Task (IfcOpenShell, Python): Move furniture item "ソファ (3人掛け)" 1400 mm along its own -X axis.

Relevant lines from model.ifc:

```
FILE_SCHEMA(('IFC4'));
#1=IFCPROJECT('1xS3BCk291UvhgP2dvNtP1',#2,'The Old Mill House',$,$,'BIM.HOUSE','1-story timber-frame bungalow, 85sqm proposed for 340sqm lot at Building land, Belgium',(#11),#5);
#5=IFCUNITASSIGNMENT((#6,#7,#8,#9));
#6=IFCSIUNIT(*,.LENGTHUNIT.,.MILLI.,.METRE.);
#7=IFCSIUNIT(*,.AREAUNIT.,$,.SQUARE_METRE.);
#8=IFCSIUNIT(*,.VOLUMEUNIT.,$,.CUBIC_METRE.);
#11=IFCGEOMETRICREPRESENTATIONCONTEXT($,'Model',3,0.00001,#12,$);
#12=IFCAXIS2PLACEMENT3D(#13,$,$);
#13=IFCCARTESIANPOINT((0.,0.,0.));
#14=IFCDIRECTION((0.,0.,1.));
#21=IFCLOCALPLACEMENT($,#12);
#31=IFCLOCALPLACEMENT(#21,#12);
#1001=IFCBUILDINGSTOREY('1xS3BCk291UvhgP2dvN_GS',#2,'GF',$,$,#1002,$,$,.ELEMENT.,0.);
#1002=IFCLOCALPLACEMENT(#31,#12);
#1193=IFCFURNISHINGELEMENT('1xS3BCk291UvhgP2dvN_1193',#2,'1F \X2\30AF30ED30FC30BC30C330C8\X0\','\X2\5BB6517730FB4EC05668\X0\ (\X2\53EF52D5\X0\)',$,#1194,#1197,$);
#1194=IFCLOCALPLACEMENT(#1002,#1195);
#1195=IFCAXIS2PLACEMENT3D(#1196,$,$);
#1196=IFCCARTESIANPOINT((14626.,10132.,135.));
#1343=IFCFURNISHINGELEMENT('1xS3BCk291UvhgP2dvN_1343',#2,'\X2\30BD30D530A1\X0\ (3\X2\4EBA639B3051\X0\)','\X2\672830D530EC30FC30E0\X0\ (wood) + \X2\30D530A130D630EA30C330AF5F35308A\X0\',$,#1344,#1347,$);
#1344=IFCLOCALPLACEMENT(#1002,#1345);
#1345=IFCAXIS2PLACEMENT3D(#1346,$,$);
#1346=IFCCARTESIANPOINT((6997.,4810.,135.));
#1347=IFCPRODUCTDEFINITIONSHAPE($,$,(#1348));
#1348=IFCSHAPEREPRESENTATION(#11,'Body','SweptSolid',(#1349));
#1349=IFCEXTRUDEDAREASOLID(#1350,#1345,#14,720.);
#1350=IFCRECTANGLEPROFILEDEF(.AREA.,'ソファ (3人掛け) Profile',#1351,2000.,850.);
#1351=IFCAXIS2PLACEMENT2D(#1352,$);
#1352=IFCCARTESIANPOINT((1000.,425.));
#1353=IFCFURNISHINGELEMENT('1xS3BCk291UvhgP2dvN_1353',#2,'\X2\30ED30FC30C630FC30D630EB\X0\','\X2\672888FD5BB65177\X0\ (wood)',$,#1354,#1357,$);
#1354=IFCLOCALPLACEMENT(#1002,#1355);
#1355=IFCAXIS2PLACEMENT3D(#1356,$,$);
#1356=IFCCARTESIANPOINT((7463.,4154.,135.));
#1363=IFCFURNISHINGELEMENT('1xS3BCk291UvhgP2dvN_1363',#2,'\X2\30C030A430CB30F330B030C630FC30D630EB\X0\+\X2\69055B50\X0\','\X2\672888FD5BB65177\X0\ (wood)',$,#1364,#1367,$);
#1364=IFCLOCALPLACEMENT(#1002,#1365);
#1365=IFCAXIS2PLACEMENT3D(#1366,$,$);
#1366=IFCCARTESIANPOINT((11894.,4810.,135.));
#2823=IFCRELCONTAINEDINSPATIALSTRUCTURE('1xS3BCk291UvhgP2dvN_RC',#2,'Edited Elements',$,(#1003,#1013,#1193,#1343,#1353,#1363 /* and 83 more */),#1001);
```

```python
import ifcopenshell
import ifcopenshell.api.geometry
import ifcopenshell.util.placement
import ifcopenshell.util.unit

model = ifcopenshell.open("model.ifc")
unit_scale = ifcopenshell.util.unit.calculate_unit_scale(model)

item = model.by_guid("1xS3BCk291UvhgP2dvN_1343")
matrix = ifcopenshell.util.placement.get_local_placement(item.ObjectPlacement)
matrix[:3, 3] -= matrix[:3, 0] * 1.4 / unit_scale
ifcopenshell.api.geometry.edit_object_placement(model, product=item, matrix=matrix, is_si=False)

print(ifcopenshell.util.placement.get_local_placement(item.ObjectPlacement).round(3) + 0.0)

model.write("model_rev.ifc")
```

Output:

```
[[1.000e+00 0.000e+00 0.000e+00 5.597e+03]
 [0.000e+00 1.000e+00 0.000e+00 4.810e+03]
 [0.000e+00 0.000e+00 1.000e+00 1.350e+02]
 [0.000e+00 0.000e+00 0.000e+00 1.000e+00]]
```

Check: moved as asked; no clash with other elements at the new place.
